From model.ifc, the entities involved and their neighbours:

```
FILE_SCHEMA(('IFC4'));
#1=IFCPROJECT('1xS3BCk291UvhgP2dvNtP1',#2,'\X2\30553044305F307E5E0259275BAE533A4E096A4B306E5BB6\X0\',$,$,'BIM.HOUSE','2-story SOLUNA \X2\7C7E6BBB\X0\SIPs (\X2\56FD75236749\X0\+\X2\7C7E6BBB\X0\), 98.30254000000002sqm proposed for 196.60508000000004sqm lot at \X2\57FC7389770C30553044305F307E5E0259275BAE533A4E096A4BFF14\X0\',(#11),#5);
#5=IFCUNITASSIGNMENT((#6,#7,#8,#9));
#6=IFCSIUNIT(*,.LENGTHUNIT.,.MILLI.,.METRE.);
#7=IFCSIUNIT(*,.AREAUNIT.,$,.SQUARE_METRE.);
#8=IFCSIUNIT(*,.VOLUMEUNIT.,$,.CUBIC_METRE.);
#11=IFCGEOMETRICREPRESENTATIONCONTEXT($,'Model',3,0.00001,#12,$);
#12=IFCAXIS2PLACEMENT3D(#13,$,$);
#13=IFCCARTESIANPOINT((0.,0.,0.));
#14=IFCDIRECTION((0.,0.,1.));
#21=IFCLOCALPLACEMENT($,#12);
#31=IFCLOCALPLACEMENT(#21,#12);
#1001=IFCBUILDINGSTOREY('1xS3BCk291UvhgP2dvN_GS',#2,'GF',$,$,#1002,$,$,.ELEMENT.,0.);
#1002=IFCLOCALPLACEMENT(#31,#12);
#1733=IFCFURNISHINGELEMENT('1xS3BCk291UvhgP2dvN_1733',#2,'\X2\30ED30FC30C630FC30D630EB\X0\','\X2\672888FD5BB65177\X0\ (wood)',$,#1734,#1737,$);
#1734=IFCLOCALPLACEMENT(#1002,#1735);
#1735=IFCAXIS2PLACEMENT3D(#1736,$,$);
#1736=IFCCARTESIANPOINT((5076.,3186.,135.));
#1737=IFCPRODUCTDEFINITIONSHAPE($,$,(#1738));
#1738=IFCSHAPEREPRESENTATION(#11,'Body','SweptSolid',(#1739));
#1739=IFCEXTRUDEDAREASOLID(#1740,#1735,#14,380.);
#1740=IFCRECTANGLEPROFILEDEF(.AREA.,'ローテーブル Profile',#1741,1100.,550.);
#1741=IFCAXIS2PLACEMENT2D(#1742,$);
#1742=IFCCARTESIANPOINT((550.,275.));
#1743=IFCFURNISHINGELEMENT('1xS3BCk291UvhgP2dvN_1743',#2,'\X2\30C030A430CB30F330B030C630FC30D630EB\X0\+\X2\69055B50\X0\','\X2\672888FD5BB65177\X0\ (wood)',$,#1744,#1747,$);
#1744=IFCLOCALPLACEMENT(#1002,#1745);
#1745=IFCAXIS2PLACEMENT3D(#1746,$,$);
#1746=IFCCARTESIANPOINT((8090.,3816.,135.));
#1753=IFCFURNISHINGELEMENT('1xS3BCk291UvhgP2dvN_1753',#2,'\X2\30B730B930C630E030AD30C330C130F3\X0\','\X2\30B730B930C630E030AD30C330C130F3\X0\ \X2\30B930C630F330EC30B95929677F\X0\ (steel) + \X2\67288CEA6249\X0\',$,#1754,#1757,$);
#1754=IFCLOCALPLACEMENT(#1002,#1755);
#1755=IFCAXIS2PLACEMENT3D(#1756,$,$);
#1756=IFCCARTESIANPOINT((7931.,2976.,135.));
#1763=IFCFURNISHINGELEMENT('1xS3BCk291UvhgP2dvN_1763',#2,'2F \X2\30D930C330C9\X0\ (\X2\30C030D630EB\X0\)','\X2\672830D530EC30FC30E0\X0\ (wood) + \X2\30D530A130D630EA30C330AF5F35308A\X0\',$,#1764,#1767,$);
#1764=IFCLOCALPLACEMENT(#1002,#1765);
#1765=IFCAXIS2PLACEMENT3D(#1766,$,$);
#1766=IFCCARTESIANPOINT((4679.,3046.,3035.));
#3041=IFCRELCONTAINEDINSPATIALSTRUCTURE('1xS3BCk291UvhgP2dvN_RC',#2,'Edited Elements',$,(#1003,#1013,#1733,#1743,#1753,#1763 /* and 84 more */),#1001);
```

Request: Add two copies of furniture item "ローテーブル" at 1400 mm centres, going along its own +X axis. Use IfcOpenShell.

```python
import ifcopenshell
import ifcopenshell.api.geometry
import ifcopenshell.api.root
import ifcopenshell.util.element
import ifcopenshell.util.placement
import ifcopenshell.util.unit

model = ifcopenshell.open("model.ifc")
unit_scale = ifcopenshell.util.unit.calculate_unit_scale(model)


def reuse_history(source, copy):
    """copy_class also copies each property set's owner history, people and application; keep the originals."""
    for rel in copy.IsDefinedBy:
        if rel.is_a("IfcRelDefinesByProperties") and (history := rel.RelatingPropertyDefinition.OwnerHistory):
            rel.RelatingPropertyDefinition.OwnerHistory = source.OwnerHistory
            ifcopenshell.util.element.remove_deep2(model, history)


source = model.by_guid("1xS3BCk291UvhgP2dvN_1733")
base = ifcopenshell.util.placement.get_local_placement(source.ObjectPlacement)
step = base[:3, 0] * 1.4 / unit_scale

for i in range(1, 3):
    copy = ifcopenshell.api.root.copy_class(model, product=source)
    copy.Representation = ifcopenshell.util.element.copy_deep(
        model, source.Representation, exclude=["IfcGeometricRepresentationContext", "IfcRepresentationMap"]
    )
    reuse_history(source, copy)
    matrix = base.copy()
    matrix[:3, 3] += i * step
    print("added at", matrix[:3, 3].round(3) + 0.0)
    ifcopenshell.api.geometry.edit_object_placement(model, product=copy, matrix=matrix, is_si=False)

model.write("model_updated.ifc")
```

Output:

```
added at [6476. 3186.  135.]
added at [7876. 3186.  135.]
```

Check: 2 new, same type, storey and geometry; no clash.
